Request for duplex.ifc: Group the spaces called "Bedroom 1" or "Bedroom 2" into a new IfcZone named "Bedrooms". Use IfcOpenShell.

First a look at what the model holds.

```python
import ifcopenshell

model = ifcopenshell.open("duplex.ifc")
print(model.schema)
seen = {}
for space in model.by_type("IfcSpace"):
    seen[space.LongName] = seen.get(space.LongName, 0) + 1
for name, count in sorted(seen.items(), key=str):
    print(count, "x", name)
print("zones:", [z.Name for z in model.by_type("IfcZone")][:20])
```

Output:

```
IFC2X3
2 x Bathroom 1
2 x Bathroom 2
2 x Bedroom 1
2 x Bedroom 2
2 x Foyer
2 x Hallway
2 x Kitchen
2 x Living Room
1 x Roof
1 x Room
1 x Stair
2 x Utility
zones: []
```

```python
import ifcopenshell
import ifcopenshell.api.group
import ifcopenshell.api.root

model = ifcopenshell.open("duplex.ifc")

names = {"Bedroom 1", "Bedroom 2"}
spaces = [s for s in model.by_type("IfcSpace") if s.LongName in names]

zone = ifcopenshell.api.root.create_entity(model, ifc_class="IfcZone", name="Bedrooms")
ifcopenshell.api.group.assign_group(model, products=spaces, group=zone)
print(len(spaces), "spaces in", zone.Name)

model.write("duplex_updated.ifc")
```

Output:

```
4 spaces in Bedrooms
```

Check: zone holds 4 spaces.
